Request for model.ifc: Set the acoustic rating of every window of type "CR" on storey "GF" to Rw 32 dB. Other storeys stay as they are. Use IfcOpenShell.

First a look at what the model holds.

```python
import ifcopenshell
import ifcopenshell.util.element

model = ifcopenshell.open("model.ifc")
print(model.schema)
storey = next(s for s in model.by_type("IfcBuildingStorey") if s.Name == "GF")
windows = [e for e in ifcopenshell.util.element.get_decomposition(storey) if e.is_a("IfcWindow")]
seen = {}
for e in windows:
    element_type = ifcopenshell.util.element.get_type(e)
    key = (element_type.Name if element_type != e and element_type else None, ifcopenshell.util.element.get_pset(e, "Pset_WindowCommon", "AcousticRating"))
    seen[key] = seen.get(key, 0) + 1
for (name, value), count in sorted(seen.items(), key=str):
    print(count, "x", name, "|", value)
```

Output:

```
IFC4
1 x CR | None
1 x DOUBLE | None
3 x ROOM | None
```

```python
import ifcopenshell
import ifcopenshell.api.pset
import ifcopenshell.util.element

model = ifcopenshell.open("model.ifc")

storey = next(s for s in model.by_type("IfcBuildingStorey") if s.Name == "GF")
windows = [e for e in ifcopenshell.util.element.get_decomposition(storey) if e.is_a("IfcWindow")]

count = 0
for e in windows:
    element_type = ifcopenshell.util.element.get_type(e)
    if element_type in (None, e) or element_type.Name != "CR":
        continue
    # add_pset returns the element's existing set when there is one.
    pset = ifcopenshell.api.pset.add_pset(model, product=e, name="Pset_WindowCommon")
    ifcopenshell.api.pset.edit_pset(model, pset=pset, properties={"AcousticRating": "Rw 32 dB"})
    count += 1

print(count, "windows updated")

model.write("model_updated.ifc")
```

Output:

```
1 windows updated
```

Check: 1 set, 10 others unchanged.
